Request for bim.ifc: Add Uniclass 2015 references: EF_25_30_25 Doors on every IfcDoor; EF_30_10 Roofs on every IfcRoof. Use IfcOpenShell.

First a look at what the model holds.

```python
import ifcopenshell

model = ifcopenshell.open("bim.ifc")
print(model.schema)
print("classifications:", [c.Name for c in model.by_type("IfcClassification")])
for ifc_class in ("IfcDoor", "IfcRoof", "IfcStair", "IfcWall", "IfcWindow"):
    print(ifc_class, len(model.by_type(ifc_class)))
```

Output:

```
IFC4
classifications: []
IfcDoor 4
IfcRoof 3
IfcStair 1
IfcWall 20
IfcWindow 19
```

```python
import ifcopenshell
import ifcopenshell.api.classification

model = ifcopenshell.open("bim.ifc")

system = ifcopenshell.api.classification.add_classification(model, classification="Uniclass 2015")

codes = {
    "IfcDoor": ("EF_25_30_25", "Doors"),
    "IfcRoof": ("EF_30_10", "Roofs"),
}
for ifc_class, (code, name) in codes.items():
    products = model.by_type(ifc_class)
    ifcopenshell.api.classification.add_reference(
        model, products=products, classification=system, identification=code, name=name
    )
    print(code, len(products))

model.write("bim_edited.ifc")
```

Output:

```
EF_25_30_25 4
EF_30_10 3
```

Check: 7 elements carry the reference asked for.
